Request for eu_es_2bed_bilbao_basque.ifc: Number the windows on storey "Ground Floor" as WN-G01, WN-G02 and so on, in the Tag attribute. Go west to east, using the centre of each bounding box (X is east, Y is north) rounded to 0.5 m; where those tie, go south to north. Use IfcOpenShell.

First a look at what the model holds.

```python
import ifcopenshell
import ifcopenshell.util.element
import ifcopenshell.util.placement

model = ifcopenshell.open("eu_es_2bed_bilbao_basque.ifc")
print(model.schema)
storey = next(s for s in model.by_type("IfcBuildingStorey") if s.Name == "Ground Floor")
windows = [e for e in ifcopenshell.util.element.get_decomposition(storey) if e.is_a("IfcWindow")]
for e in sorted(windows, key=lambda e: e.id()):
    origin = ifcopenshell.util.placement.get_local_placement(e.ObjectPlacement)[:3, 3]
    print(e.id(), e.Tag, e.Name, origin.round(2) + 0.0, sep=" | ")
```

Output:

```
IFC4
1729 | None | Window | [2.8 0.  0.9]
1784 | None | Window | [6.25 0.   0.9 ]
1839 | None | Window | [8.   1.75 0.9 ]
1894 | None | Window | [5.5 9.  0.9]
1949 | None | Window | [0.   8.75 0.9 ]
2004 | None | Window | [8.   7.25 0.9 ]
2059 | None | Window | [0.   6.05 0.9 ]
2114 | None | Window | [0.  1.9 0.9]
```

```python
import ifcopenshell
import ifcopenshell.geom
import ifcopenshell.util.element
import ifcopenshell.util.shape

model = ifcopenshell.open("eu_es_2bed_bilbao_basque.ifc")
settings = ifcopenshell.geom.settings()
settings.set("use-world-coords", True)


def centre(element):
    shape = ifcopenshell.geom.create_shape(settings, element)
    return ifcopenshell.util.shape.get_bbox_centroid(shape.geometry)


storey = next(s for s in model.by_type("IfcBuildingStorey") if s.Name == "Ground Floor")
windows = [e for e in ifcopenshell.util.element.get_decomposition(storey) if e.is_a("IfcWindow")]

# Insertion points can sit at a corner or the storey origin, so sort by the geometry (in metres).
centres = {e: centre(e) for e in windows}
windows.sort(key=lambda e: (round(centres[e][0] / 0.5), centres[e][1]))

for i, e in enumerate(windows, start=1):
    number = f"WN-G{i:02d}"
    e.Tag = number
    print(e.id(), number)

model.write("eu_es_2bed_bilbao_basque_updated.ifc")
```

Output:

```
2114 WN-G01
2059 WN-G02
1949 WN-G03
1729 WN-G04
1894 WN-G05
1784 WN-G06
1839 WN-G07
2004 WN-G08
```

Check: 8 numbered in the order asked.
